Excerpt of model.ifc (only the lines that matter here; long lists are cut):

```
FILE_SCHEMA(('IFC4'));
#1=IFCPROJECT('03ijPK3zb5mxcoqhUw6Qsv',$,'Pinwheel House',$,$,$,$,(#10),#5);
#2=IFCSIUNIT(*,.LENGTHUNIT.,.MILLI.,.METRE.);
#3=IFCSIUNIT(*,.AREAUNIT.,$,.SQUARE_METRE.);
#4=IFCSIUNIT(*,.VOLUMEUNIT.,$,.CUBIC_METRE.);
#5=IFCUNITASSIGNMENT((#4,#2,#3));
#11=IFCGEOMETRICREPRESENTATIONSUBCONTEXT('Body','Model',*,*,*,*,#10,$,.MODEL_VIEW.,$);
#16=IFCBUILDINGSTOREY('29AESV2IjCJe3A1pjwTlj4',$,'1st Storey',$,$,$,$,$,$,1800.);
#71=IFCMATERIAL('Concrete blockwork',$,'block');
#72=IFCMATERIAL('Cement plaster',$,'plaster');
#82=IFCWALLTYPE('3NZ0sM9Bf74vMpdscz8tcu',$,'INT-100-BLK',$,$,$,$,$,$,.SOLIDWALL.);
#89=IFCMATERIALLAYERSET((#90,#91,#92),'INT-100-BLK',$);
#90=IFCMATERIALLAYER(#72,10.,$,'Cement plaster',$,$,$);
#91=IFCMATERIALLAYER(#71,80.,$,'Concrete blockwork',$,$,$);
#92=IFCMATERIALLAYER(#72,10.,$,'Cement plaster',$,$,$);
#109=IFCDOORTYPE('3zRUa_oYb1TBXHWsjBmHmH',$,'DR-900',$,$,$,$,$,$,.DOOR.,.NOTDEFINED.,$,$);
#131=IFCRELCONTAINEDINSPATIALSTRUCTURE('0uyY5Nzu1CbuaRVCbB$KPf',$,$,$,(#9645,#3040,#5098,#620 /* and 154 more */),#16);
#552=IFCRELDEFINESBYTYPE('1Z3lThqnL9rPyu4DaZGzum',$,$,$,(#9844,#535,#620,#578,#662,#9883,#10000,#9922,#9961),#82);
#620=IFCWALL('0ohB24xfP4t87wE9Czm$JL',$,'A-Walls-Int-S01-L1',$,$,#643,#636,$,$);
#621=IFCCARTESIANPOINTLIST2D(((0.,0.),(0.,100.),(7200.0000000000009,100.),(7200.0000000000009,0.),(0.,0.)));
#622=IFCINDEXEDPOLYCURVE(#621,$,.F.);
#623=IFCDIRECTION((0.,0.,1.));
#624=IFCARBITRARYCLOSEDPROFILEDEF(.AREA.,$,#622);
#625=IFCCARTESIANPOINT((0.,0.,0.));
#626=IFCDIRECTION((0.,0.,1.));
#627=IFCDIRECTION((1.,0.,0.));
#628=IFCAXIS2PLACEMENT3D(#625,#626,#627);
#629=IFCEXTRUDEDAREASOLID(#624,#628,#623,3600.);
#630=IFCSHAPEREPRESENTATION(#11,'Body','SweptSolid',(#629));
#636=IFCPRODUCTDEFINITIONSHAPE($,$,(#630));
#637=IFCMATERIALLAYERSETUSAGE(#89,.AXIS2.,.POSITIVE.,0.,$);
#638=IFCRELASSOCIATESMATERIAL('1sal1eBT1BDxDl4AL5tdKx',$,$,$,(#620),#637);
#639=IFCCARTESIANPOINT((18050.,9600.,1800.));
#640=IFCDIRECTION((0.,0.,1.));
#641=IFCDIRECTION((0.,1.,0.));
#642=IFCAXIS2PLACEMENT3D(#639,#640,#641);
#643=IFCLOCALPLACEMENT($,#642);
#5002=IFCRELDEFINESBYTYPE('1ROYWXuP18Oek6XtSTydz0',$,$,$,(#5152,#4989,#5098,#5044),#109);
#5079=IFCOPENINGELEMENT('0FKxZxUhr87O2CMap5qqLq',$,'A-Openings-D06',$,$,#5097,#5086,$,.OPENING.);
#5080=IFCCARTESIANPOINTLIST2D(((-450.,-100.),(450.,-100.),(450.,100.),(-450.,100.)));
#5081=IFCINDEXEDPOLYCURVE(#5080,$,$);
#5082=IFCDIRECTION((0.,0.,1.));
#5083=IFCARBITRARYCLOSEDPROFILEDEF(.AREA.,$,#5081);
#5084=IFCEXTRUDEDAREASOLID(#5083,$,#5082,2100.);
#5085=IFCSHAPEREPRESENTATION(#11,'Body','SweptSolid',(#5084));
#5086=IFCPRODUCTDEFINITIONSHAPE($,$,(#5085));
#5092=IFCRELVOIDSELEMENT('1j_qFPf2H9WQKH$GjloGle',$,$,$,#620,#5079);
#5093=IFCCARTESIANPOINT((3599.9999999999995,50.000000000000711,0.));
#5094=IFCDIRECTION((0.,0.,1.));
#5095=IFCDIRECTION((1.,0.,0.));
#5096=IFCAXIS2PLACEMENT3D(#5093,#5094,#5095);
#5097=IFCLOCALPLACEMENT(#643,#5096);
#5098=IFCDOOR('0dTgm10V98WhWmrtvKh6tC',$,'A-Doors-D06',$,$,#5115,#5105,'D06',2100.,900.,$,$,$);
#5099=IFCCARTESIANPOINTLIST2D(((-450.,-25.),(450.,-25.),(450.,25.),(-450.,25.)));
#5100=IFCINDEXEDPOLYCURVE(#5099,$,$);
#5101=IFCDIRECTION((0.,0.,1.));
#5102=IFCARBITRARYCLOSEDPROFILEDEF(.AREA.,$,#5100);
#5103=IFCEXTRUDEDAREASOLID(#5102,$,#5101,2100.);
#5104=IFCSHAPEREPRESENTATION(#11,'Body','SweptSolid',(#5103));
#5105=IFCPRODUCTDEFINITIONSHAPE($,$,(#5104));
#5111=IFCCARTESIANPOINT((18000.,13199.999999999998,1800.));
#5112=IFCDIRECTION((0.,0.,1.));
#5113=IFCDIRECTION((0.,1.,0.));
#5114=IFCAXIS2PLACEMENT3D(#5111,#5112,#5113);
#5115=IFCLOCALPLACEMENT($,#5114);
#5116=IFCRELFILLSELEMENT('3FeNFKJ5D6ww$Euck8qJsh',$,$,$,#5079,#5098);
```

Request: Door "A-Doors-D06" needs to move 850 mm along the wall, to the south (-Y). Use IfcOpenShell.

```python
import ifcopenshell
import ifcopenshell.api.geometry
import ifcopenshell.util.placement
import ifcopenshell.util.unit

model = ifcopenshell.open("model.ifc")
unit_scale = ifcopenshell.util.unit.calculate_unit_scale(model)

door = model.by_guid("0dTgm10V98WhWmrtvKh6tC")
opening = door.FillsVoids[0].RelatingOpeningElement
wall = opening.VoidsElements[0].RelatingBuildingElement

wall_matrix = ifcopenshell.util.placement.get_local_placement(wall.ObjectPlacement)
shift = wall_matrix[:3, 0] * -0.85 / unit_scale
before = ifcopenshell.util.placement.get_local_placement(door.ObjectPlacement)[:3, 3].copy()

# The door is not placed relative to its opening, so move both.
for product in (opening, door):
    matrix = ifcopenshell.util.placement.get_local_placement(product.ObjectPlacement)
    matrix[:3, 3] += shift
    ifcopenshell.api.geometry.edit_object_placement(model, product=product, matrix=matrix, is_si=False)

after = ifcopenshell.util.placement.get_local_placement(door.ObjectPlacement)[:3, 3]
print("door moved by", (after - before).round(3) + 0.0)

model.write("model_updated.ifc")
```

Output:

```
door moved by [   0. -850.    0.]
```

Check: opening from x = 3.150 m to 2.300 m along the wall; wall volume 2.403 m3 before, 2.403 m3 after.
